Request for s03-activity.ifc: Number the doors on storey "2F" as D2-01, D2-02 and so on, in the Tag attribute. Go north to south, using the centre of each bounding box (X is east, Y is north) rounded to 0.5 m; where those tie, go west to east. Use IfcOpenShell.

First a look at what the model holds.

```python
import ifcopenshell
import ifcopenshell.util.element
import ifcopenshell.util.placement

model = ifcopenshell.open("s03-activity.ifc")
print(model.schema)
storey = next(s for s in model.by_type("IfcBuildingStorey") if s.Name == "2F")
doors = [e for e in ifcopenshell.util.element.get_decomposition(storey) if e.is_a("IfcDoor")]
for e in sorted(doors, key=lambda e: e.id()):
    origin = ifcopenshell.util.placement.get_local_placement(e.ObjectPlacement)[:3, 3]
    print(e.id(), e.Tag, e.Name, origin.round(2) + 0.0, sep=" | ")
```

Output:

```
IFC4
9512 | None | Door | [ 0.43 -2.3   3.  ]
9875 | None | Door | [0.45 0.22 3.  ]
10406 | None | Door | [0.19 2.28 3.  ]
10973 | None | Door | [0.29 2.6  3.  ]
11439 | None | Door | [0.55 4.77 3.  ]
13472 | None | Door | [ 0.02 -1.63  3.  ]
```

```python
import ifcopenshell
import ifcopenshell.geom
import ifcopenshell.util.element
import ifcopenshell.util.shape

model = ifcopenshell.open("s03-activity.ifc")
settings = ifcopenshell.geom.settings()
settings.set("use-world-coords", True)


def centre(element):
    shape = ifcopenshell.geom.create_shape(settings, element)
    return ifcopenshell.util.shape.get_bbox_centroid(shape.geometry)


storey = next(s for s in model.by_type("IfcBuildingStorey") if s.Name == "2F")
doors = [e for e in ifcopenshell.util.element.get_decomposition(storey) if e.is_a("IfcDoor")]

# Insertion points can sit at a corner or the storey origin, so sort by the geometry (in metres).
centres = {e: centre(e) for e in doors}
doors.sort(key=lambda e: (-round(centres[e][1] / 0.5), centres[e][0]))

for i, e in enumerate(doors, start=1):
    number = f"D2-{i:02d}"
    e.Tag = number
    print(e.id(), number)

model.write("s03-activity_updated.ifc")
```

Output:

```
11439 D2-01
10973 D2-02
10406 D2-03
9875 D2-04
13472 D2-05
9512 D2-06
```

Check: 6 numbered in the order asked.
